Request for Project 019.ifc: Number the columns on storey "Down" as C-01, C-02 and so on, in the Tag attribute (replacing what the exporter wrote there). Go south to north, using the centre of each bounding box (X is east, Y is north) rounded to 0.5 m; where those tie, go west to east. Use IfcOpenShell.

First a look at what the model holds.

```python
import ifcopenshell
import ifcopenshell.util.element
import ifcopenshell.util.placement

model = ifcopenshell.open("Project 019.ifc")
print(model.schema)
storey = next(s for s in model.by_type("IfcBuildingStorey") if s.Name == "Down")
columns = [e for e in ifcopenshell.util.element.get_decomposition(storey) if e.is_a("IfcColumn")]
for e in sorted(columns, key=lambda e: e.id()):
    origin = ifcopenshell.util.placement.get_local_placement(e.ObjectPlacement)[:3, 3]
    print(e.id(), e.Tag, e.Name, origin.round(2) + 0.0, sep=" | ")
```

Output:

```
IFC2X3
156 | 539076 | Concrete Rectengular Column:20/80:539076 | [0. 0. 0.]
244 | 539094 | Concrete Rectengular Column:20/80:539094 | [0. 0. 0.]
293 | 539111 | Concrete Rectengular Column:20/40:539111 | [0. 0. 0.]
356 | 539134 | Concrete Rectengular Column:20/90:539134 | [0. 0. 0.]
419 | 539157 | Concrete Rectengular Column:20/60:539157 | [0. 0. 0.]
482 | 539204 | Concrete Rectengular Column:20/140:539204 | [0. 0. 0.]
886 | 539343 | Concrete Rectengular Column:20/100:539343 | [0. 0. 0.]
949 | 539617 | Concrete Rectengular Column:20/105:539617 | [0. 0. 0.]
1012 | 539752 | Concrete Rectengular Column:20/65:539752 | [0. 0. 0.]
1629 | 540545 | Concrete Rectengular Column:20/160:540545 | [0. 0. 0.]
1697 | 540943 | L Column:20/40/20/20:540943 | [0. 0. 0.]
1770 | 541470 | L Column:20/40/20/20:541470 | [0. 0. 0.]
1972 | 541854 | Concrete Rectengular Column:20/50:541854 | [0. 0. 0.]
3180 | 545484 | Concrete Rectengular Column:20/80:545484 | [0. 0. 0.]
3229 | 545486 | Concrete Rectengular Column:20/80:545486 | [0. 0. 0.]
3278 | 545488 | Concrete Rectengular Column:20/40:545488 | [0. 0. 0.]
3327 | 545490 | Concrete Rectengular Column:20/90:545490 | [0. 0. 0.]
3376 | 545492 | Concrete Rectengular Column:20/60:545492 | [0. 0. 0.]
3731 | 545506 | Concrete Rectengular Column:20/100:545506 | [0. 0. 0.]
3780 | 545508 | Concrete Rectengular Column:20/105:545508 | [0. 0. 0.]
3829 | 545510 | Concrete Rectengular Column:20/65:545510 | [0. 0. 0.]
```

```python
import ifcopenshell
import ifcopenshell.geom
import ifcopenshell.util.element
import ifcopenshell.util.shape

model = ifcopenshell.open("Project 019.ifc")
settings = ifcopenshell.geom.settings()
settings.set("use-world-coords", True)


def centre(element):
    shape = ifcopenshell.geom.create_shape(settings, element)
    return ifcopenshell.util.shape.get_bbox_centroid(shape.geometry)


storey = next(s for s in model.by_type("IfcBuildingStorey") if s.Name == "Down")
columns = [e for e in ifcopenshell.util.element.get_decomposition(storey) if e.is_a("IfcColumn")]

# Insertion points can sit at a corner or the storey origin, so sort by the geometry (in metres).
centres = {e: centre(e) for e in columns}
columns.sort(key=lambda e: (round(centres[e][1] / 0.5), centres[e][0]))

for i, e in enumerate(columns, start=1):
    number = f"C-{i:02d}"
    e.Tag = number
    print(e.id(), number)

model.write("Project 019_updated.ifc")
```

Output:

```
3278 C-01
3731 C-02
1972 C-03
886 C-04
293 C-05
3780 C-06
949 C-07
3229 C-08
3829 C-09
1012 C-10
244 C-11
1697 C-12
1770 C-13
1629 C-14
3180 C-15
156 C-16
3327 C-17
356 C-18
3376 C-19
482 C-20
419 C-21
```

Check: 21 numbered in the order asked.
